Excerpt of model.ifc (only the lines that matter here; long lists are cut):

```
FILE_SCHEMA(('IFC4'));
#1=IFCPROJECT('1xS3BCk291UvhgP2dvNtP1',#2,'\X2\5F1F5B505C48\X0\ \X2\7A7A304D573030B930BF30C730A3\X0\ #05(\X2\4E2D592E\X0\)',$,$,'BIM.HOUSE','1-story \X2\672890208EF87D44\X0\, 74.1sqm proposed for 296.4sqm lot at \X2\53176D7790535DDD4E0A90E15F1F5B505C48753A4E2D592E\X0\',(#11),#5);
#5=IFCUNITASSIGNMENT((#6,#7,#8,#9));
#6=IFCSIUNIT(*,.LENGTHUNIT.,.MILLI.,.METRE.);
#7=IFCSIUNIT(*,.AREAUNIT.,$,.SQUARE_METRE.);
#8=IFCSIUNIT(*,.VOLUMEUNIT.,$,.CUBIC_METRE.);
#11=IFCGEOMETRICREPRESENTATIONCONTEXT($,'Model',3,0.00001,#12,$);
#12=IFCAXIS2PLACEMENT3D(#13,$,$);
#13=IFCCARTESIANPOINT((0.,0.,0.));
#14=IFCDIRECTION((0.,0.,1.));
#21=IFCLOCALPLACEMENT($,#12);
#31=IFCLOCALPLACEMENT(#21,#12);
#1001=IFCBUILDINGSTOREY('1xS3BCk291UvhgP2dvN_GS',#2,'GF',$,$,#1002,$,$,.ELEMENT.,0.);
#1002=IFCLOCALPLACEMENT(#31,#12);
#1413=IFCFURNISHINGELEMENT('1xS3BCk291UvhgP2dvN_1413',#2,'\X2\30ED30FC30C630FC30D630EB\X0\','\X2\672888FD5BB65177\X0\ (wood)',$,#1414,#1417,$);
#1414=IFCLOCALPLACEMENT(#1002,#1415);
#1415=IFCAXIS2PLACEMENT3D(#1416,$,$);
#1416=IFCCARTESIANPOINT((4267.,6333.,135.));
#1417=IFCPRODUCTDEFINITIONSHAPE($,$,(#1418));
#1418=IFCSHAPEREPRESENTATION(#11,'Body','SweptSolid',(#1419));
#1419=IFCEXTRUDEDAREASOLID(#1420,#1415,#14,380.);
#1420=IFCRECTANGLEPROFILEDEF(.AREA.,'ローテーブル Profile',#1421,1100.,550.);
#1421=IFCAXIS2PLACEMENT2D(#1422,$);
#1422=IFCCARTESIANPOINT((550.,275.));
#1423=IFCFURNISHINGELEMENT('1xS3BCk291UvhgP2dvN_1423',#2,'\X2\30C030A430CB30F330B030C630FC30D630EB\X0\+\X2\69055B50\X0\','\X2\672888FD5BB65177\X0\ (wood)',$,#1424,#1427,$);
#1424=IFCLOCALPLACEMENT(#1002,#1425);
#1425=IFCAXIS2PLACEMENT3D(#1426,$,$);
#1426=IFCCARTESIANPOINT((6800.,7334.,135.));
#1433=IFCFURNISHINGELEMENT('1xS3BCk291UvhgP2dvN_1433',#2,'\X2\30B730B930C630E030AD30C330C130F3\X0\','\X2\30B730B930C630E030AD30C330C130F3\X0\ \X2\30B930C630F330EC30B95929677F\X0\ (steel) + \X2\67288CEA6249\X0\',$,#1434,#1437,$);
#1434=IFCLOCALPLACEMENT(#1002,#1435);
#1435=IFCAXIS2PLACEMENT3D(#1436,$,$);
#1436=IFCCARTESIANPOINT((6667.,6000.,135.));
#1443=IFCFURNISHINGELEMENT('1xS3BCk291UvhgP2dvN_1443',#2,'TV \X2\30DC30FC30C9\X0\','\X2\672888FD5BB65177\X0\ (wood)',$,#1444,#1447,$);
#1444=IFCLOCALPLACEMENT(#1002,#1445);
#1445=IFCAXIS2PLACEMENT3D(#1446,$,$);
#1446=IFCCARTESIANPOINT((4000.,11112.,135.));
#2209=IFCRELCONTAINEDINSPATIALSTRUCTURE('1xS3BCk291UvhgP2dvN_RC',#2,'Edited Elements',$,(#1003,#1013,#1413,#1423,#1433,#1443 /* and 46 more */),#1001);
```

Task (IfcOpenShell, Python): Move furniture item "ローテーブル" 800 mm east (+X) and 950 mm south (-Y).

```python
import ifcopenshell
import ifcopenshell.api.geometry
import ifcopenshell.util.placement

model = ifcopenshell.open("model.ifc")

item = model.by_guid("1xS3BCk291UvhgP2dvN_1413")
matrix = ifcopenshell.util.placement.get_local_placement(item.ObjectPlacement)
matrix[0, 3] += 800.0
matrix[1, 3] -= 950.0
ifcopenshell.api.geometry.edit_object_placement(model, product=item, matrix=matrix, is_si=False)

print(ifcopenshell.util.placement.get_local_placement(item.ObjectPlacement).round(3) + 0.0)

model.write("model_edited.ifc")
```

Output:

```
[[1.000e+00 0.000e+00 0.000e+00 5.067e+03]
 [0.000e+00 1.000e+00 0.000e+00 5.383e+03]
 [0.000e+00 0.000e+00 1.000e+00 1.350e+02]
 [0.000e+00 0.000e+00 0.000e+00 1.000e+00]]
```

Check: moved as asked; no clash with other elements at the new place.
